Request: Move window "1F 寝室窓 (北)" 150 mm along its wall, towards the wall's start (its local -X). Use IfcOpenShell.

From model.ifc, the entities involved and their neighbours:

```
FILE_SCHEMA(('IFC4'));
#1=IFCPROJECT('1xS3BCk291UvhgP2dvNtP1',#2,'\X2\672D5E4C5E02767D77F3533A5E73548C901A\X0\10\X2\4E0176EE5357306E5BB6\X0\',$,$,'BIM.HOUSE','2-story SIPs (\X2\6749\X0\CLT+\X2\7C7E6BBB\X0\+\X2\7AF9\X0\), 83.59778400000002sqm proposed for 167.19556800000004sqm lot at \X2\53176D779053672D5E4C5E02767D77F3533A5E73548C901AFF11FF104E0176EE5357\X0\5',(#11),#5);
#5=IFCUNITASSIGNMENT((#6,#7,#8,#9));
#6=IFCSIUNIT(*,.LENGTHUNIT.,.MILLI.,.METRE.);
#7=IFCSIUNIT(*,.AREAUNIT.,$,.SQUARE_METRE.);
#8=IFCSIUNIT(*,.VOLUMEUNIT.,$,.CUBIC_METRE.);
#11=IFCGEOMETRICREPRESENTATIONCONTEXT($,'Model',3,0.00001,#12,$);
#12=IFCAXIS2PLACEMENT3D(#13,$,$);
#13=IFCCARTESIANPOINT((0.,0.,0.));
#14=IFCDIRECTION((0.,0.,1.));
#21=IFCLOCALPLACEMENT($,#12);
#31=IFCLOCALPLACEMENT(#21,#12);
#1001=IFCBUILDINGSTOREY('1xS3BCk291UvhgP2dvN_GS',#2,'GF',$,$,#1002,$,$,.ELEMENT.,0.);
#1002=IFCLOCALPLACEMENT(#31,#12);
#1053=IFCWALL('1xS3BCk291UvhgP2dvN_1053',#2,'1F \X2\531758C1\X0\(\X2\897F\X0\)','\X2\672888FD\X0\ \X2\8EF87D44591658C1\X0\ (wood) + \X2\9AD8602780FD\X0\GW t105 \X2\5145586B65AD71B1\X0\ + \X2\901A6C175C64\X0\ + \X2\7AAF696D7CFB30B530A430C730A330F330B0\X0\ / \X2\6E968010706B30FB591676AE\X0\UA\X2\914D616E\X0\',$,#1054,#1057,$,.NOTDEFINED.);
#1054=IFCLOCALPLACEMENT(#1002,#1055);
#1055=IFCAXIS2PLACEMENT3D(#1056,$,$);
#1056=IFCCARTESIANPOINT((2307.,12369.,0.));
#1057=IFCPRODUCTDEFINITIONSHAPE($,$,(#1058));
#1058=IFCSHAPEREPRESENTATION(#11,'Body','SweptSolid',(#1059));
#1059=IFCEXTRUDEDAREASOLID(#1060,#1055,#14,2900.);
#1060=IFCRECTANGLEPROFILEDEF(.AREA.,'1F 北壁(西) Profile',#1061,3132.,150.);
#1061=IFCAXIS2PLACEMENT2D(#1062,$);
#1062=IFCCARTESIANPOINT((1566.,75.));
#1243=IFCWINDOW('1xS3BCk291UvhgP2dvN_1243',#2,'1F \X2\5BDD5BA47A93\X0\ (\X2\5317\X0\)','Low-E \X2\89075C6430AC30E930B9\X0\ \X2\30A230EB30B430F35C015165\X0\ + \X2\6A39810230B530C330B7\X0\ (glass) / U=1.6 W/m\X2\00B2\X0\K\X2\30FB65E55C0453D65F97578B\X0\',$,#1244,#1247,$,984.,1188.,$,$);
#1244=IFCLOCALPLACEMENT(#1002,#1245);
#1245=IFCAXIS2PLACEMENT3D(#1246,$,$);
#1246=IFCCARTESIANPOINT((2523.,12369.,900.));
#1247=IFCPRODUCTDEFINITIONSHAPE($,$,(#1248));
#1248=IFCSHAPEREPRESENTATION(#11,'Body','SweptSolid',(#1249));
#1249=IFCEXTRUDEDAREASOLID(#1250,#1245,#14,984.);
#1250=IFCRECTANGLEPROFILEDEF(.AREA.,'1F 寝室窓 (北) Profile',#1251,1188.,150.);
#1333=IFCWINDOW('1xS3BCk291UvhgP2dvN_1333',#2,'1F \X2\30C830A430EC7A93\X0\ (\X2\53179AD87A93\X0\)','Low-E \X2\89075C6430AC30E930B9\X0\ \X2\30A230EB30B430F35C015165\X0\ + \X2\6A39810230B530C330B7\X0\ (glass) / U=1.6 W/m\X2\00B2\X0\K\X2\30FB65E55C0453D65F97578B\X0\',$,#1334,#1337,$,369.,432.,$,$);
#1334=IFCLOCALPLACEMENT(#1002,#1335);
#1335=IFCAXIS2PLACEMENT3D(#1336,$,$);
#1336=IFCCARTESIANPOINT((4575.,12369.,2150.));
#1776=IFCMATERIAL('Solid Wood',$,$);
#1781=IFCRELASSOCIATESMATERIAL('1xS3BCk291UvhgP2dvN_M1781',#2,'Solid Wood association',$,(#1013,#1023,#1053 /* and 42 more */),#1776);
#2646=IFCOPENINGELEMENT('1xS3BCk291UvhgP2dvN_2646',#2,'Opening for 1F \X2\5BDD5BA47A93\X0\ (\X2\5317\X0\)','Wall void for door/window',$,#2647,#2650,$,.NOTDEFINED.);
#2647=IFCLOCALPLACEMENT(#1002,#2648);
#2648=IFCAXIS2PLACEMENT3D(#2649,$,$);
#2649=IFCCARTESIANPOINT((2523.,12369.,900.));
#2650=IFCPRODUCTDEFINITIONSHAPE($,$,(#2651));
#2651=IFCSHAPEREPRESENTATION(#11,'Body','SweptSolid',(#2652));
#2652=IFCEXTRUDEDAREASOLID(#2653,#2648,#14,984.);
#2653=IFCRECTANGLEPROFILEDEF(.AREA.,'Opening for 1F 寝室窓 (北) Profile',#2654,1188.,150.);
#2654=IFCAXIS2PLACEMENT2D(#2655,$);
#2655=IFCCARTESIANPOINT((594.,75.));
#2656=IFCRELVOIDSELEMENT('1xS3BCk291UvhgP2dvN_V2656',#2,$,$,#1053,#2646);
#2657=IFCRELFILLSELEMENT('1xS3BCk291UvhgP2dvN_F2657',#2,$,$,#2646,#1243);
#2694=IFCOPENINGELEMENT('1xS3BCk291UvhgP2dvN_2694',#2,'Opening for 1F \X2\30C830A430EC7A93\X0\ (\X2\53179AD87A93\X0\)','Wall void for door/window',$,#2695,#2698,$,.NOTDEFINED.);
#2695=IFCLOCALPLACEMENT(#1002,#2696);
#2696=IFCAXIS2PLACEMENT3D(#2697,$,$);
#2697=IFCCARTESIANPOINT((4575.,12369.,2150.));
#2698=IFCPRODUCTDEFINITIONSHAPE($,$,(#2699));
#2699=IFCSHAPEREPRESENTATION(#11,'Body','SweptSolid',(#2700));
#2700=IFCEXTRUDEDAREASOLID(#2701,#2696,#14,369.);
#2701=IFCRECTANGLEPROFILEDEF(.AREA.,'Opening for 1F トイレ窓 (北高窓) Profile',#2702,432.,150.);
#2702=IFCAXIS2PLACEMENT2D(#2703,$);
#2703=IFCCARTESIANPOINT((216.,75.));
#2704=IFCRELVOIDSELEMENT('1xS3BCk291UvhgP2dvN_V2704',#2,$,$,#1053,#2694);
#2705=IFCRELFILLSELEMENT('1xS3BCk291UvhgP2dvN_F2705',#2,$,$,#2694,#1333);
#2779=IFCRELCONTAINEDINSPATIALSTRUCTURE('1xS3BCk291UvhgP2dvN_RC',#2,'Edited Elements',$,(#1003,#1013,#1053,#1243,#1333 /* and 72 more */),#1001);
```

```python
import ifcopenshell
import ifcopenshell.api.geometry
import ifcopenshell.util.placement

model = ifcopenshell.open("model.ifc")

window = model.by_guid("1xS3BCk291UvhgP2dvN_1243")
opening = window.FillsVoids[0].RelatingOpeningElement
wall = opening.VoidsElements[0].RelatingBuildingElement

wall_matrix = ifcopenshell.util.placement.get_local_placement(wall.ObjectPlacement)
shift = wall_matrix[:3, 0] * -150.0
before = ifcopenshell.util.placement.get_local_placement(window.ObjectPlacement)[:3, 3].copy()

# The window is not placed relative to its opening, so move both.
for product in (opening, window):
    matrix = ifcopenshell.util.placement.get_local_placement(product.ObjectPlacement)
    matrix[:3, 3] += shift
    ifcopenshell.api.geometry.edit_object_placement(model, product=product, matrix=matrix, is_si=False)

after = ifcopenshell.util.placement.get_local_placement(window.ObjectPlacement)[:3, 3]
print("window moved by", (after - before).round(3) + 0.0)

model.write("model_updated.ifc")
```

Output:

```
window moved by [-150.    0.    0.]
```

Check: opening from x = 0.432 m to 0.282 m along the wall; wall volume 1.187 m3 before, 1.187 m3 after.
